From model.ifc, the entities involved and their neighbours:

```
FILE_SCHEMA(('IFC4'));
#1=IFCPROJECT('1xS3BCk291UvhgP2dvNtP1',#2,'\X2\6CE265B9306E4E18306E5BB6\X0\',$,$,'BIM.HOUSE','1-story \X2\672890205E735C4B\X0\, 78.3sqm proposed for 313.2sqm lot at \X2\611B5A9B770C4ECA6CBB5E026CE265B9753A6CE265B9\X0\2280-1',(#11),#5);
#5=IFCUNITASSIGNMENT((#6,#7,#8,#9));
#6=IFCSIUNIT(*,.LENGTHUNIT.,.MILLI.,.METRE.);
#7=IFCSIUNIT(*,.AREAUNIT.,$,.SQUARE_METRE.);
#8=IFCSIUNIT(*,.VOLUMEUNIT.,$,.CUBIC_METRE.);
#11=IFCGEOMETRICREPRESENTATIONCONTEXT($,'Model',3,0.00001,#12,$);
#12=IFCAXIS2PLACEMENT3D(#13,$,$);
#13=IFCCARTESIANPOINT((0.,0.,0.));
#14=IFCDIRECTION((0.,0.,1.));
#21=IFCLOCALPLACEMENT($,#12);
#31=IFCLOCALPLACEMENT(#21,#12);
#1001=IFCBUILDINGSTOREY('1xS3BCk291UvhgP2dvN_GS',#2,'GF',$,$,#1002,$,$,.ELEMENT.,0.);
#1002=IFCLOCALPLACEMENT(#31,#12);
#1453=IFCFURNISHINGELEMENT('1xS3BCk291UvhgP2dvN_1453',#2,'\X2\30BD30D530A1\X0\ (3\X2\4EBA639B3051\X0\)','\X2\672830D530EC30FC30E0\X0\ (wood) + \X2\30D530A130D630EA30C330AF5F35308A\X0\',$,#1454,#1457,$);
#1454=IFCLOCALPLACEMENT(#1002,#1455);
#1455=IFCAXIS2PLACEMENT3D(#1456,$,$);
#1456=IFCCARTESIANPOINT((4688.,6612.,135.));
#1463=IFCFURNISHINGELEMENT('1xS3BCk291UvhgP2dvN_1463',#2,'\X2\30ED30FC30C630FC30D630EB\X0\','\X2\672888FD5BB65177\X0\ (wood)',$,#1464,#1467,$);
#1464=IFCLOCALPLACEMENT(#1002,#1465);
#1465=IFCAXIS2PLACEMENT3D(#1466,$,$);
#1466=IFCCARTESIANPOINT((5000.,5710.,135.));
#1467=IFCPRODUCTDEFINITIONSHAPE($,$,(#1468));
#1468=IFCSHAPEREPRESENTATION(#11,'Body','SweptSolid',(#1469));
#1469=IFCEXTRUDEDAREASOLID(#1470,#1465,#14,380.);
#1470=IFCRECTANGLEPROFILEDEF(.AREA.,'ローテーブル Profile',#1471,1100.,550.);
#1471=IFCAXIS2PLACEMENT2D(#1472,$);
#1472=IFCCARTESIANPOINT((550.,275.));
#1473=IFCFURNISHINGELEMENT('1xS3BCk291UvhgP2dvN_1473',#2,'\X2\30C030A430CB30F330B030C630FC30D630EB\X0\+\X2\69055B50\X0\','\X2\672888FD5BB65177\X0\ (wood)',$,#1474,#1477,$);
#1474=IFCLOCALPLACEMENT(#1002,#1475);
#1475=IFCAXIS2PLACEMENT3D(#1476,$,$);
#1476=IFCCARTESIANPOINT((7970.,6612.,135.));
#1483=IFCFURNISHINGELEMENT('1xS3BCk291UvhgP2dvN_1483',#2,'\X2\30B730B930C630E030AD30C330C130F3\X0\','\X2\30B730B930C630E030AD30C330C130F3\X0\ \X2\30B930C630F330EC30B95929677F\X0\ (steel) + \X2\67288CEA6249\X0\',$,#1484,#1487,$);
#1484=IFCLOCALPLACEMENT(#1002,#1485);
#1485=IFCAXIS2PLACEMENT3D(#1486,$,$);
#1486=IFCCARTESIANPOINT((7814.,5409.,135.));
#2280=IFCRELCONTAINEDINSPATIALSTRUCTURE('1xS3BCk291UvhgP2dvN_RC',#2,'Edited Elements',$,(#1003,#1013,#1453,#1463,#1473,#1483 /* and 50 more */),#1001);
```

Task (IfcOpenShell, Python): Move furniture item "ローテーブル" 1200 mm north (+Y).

```python
import ifcopenshell
import ifcopenshell.api.geometry
import ifcopenshell.util.placement

model = ifcopenshell.open("model.ifc")

item = model.by_id(1463)
matrix = ifcopenshell.util.placement.get_local_placement(item.ObjectPlacement)
matrix[1, 3] += 1200.0
ifcopenshell.api.geometry.edit_object_placement(model, product=item, matrix=matrix, is_si=False)

print(ifcopenshell.util.placement.get_local_placement(item.ObjectPlacement).round(3) + 0.0)

model.write("model-out.ifc")
```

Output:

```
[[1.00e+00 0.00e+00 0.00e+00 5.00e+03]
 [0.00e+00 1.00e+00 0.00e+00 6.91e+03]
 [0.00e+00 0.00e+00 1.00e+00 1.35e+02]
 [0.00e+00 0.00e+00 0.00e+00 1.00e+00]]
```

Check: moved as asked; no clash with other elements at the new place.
